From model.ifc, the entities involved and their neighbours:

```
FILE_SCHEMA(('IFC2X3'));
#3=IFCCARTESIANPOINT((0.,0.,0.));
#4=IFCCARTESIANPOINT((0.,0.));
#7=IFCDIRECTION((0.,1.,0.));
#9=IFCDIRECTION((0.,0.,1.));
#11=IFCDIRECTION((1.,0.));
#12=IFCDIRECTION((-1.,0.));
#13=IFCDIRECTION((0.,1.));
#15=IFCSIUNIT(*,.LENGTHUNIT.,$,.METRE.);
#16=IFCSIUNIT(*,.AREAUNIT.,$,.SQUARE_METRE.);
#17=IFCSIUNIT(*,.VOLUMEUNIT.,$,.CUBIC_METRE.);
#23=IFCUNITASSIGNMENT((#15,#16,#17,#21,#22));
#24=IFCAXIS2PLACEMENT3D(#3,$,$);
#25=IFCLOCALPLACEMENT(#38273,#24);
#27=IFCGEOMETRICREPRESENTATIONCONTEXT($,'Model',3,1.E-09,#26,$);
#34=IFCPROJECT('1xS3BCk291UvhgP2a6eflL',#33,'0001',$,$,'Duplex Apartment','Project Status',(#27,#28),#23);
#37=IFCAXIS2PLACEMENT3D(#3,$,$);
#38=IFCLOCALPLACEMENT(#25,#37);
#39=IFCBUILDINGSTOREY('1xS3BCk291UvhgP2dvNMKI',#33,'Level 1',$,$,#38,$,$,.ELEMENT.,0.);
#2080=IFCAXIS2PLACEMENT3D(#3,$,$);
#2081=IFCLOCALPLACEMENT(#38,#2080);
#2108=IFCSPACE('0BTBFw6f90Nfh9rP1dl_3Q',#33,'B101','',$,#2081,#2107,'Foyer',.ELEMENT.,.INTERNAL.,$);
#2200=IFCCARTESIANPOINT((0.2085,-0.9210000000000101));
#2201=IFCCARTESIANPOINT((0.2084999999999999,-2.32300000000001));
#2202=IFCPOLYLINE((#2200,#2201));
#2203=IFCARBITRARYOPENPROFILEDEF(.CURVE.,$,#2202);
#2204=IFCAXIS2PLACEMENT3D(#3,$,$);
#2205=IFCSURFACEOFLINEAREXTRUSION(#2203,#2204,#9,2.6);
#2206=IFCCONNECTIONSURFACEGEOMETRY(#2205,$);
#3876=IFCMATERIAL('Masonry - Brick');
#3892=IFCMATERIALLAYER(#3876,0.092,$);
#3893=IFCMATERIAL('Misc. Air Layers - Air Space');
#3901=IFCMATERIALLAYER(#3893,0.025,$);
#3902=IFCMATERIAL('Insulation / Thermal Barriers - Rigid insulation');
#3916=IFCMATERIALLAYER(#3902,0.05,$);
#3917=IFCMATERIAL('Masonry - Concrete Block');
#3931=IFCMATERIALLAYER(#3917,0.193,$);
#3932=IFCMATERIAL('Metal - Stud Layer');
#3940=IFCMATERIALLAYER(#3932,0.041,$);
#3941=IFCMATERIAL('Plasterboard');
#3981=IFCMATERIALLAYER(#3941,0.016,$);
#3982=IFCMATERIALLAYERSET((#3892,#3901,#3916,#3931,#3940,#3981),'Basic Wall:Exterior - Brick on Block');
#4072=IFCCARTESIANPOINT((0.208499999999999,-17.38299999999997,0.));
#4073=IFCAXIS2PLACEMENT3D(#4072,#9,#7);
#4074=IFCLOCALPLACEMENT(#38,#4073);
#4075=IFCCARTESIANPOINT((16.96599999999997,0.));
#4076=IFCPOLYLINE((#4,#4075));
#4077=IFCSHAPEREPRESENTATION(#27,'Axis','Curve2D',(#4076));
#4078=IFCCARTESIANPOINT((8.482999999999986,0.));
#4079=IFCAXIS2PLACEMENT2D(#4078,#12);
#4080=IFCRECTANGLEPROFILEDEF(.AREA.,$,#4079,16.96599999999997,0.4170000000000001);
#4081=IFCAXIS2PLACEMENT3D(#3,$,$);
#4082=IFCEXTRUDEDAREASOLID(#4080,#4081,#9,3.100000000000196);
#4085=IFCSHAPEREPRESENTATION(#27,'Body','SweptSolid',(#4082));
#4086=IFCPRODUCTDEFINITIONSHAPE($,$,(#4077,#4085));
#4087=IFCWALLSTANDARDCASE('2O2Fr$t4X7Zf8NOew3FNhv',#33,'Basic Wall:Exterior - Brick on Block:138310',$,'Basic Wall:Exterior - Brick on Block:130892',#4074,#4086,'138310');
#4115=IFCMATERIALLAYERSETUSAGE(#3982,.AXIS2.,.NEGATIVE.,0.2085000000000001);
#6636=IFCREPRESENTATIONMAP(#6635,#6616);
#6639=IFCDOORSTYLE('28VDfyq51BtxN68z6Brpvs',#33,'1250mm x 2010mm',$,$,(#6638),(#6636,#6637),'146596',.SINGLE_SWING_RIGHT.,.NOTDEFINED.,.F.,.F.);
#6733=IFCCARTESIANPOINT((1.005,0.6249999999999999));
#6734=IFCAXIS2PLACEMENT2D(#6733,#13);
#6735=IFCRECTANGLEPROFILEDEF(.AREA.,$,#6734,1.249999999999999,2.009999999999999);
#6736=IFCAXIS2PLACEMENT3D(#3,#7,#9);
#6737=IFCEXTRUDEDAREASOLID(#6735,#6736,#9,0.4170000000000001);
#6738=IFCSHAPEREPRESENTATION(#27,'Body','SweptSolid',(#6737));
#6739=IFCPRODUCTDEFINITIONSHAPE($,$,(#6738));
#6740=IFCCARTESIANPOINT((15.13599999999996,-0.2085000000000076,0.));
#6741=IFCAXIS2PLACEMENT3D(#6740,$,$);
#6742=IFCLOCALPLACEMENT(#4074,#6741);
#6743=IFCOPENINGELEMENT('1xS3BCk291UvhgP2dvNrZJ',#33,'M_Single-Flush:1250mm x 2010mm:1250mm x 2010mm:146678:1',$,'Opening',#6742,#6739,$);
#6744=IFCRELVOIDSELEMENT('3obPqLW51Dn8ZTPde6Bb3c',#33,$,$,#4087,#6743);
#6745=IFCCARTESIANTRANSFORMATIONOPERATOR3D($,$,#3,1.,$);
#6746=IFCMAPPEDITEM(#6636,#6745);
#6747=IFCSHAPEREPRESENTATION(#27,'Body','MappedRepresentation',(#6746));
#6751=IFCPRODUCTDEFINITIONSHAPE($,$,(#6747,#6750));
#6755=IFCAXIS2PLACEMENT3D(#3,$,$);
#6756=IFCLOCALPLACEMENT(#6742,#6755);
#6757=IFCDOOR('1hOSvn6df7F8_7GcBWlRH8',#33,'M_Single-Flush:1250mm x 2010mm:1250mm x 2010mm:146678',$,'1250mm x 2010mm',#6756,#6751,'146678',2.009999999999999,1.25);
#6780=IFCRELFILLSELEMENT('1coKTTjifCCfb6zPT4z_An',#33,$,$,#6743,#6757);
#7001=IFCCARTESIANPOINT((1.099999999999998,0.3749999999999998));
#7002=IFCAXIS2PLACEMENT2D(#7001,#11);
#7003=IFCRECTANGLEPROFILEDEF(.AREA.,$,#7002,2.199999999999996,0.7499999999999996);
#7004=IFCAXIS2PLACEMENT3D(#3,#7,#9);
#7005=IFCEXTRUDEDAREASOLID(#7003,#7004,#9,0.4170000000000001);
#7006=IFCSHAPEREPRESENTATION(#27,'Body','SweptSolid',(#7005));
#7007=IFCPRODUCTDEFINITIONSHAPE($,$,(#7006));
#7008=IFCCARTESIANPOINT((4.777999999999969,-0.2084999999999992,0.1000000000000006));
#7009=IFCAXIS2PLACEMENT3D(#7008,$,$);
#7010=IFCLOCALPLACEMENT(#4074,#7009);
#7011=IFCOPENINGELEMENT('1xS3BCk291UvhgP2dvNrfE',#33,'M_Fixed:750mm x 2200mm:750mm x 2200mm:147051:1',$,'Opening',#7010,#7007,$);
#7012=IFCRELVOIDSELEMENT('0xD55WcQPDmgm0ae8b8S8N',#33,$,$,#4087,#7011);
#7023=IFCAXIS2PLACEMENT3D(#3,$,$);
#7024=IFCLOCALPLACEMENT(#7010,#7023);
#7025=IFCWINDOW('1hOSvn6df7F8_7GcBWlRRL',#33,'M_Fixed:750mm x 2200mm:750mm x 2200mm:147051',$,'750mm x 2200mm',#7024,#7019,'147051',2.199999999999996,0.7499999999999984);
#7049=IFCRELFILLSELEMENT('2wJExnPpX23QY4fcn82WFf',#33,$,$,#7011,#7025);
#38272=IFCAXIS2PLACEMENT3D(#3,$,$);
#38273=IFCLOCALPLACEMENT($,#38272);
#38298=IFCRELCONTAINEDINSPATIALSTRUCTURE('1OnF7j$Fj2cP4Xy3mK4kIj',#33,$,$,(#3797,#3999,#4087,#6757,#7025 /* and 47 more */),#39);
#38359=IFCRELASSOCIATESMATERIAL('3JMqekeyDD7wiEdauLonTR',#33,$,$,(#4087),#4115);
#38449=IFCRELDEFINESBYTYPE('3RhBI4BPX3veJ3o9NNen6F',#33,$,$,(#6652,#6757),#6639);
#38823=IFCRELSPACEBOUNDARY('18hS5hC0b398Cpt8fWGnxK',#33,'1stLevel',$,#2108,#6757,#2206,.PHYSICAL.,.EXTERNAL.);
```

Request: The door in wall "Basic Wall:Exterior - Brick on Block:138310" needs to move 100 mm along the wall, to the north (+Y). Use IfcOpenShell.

```python
import numpy as np
import ifcopenshell
import ifcopenshell.api.geometry
import ifcopenshell.util.placement
import ifcopenshell.util.unit

model = ifcopenshell.open("model.ifc")
unit_scale = ifcopenshell.util.unit.calculate_unit_scale(model)

door = model.by_id(6757)
opening = door.FillsVoids[0].RelatingOpeningElement
wall = opening.VoidsElements[0].RelatingBuildingElement

wall_matrix = ifcopenshell.util.placement.get_local_placement(wall.ObjectPlacement)
shift = wall_matrix[:3, 0] * 0.1 / unit_scale
before = ifcopenshell.util.placement.get_local_placement(door.ObjectPlacement)[:3, 3].copy()

# The door is placed relative to its opening, so it follows when the opening moves.
matrix = ifcopenshell.util.placement.get_local_placement(opening.ObjectPlacement)
matrix[:3, 3] += shift
ifcopenshell.api.geometry.edit_object_placement(
    model, product=opening, matrix=matrix, is_si=False, should_transform_children=True
)

# Space boundary surfaces are stored in each space's coordinates; move them too.
for rel in door.ProvidesBoundaries:
    if not rel.ConnectionGeometry:
        continue
    surface = rel.ConnectionGeometry.SurfaceOnRelatingElement
    space_matrix = ifcopenshell.util.placement.get_local_placement(rel.RelatingSpace.ObjectPlacement)
    point = np.array(surface.Position.Location.Coordinates) + space_matrix[:3, :3].T @ shift
    surface.Position = model.createIfcAxis2Placement3D(
        model.createIfcCartesianPoint(point.tolist()), surface.Position.Axis, surface.Position.RefDirection
    )

after = ifcopenshell.util.placement.get_local_placement(door.ObjectPlacement)[:3, 3]
print("door moved by", (after - before).round(3) + 0.0)

model.write("model_edited.ifc")
```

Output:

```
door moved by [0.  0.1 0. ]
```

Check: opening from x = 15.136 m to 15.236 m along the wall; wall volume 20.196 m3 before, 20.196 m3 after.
